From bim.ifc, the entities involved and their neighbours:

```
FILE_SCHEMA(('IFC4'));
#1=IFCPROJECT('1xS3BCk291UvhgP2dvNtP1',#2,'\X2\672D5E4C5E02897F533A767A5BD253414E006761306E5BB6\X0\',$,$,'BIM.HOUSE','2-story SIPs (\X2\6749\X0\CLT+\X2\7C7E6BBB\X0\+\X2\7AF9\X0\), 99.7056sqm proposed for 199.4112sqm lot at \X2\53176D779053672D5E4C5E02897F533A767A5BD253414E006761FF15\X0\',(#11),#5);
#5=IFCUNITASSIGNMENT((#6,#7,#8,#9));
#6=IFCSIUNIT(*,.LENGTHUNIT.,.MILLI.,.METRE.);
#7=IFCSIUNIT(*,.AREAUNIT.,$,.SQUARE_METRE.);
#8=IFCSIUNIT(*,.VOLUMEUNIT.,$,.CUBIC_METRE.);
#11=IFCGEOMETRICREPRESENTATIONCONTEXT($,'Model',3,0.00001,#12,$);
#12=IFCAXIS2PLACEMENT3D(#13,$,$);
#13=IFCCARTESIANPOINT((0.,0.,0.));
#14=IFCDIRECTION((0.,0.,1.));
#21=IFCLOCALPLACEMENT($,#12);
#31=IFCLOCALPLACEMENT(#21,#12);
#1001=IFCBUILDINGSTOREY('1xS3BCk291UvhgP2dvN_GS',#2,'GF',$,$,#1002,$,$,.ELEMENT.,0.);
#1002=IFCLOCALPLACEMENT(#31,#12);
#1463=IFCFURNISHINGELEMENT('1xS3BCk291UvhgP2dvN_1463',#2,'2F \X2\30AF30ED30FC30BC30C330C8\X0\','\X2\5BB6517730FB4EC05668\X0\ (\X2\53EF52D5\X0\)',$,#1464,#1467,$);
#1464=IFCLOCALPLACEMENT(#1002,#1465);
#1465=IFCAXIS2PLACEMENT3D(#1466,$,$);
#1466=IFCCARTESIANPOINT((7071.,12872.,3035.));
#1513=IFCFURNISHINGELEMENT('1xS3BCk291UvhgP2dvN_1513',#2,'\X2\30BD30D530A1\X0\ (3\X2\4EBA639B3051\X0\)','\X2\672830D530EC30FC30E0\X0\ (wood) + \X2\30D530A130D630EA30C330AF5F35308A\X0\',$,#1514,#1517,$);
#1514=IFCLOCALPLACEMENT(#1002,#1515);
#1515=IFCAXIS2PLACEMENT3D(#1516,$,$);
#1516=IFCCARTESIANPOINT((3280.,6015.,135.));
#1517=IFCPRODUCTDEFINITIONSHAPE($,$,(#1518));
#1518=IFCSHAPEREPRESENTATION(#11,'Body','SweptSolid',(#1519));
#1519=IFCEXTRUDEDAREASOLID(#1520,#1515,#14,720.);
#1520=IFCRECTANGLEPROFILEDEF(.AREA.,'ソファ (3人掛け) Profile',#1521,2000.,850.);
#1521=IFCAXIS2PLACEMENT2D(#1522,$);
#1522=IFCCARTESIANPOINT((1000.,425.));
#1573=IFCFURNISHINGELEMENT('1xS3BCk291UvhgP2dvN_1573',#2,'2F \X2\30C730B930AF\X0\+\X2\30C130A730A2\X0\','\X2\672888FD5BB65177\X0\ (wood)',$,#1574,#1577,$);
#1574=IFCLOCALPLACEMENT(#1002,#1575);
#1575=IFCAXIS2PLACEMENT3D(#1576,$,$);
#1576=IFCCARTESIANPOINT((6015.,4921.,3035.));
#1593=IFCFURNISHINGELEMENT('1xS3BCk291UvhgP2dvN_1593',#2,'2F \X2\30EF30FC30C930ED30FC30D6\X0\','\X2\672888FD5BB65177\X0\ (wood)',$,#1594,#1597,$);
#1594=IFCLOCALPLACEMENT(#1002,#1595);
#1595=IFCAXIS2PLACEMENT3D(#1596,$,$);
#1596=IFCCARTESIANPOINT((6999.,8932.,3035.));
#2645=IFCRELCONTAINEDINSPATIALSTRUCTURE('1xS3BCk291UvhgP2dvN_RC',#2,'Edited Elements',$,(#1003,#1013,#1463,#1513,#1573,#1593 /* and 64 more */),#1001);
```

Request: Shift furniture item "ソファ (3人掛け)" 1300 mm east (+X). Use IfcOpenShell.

```python
import ifcopenshell
import ifcopenshell.api.geometry
import ifcopenshell.util.placement

model = ifcopenshell.open("bim.ifc")

item = model.by_id(1513)
matrix = ifcopenshell.util.placement.get_local_placement(item.ObjectPlacement)
matrix[0, 3] += 1300.0
ifcopenshell.api.geometry.edit_object_placement(model, product=item, matrix=matrix, is_si=False)

print(ifcopenshell.util.placement.get_local_placement(item.ObjectPlacement).round(3) + 0.0)

model.write("bim-out.ifc")
```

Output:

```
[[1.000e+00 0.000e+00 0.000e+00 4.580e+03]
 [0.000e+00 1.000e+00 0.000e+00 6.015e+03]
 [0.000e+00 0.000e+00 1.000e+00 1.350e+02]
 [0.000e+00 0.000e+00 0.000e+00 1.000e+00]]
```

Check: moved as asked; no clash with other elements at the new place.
